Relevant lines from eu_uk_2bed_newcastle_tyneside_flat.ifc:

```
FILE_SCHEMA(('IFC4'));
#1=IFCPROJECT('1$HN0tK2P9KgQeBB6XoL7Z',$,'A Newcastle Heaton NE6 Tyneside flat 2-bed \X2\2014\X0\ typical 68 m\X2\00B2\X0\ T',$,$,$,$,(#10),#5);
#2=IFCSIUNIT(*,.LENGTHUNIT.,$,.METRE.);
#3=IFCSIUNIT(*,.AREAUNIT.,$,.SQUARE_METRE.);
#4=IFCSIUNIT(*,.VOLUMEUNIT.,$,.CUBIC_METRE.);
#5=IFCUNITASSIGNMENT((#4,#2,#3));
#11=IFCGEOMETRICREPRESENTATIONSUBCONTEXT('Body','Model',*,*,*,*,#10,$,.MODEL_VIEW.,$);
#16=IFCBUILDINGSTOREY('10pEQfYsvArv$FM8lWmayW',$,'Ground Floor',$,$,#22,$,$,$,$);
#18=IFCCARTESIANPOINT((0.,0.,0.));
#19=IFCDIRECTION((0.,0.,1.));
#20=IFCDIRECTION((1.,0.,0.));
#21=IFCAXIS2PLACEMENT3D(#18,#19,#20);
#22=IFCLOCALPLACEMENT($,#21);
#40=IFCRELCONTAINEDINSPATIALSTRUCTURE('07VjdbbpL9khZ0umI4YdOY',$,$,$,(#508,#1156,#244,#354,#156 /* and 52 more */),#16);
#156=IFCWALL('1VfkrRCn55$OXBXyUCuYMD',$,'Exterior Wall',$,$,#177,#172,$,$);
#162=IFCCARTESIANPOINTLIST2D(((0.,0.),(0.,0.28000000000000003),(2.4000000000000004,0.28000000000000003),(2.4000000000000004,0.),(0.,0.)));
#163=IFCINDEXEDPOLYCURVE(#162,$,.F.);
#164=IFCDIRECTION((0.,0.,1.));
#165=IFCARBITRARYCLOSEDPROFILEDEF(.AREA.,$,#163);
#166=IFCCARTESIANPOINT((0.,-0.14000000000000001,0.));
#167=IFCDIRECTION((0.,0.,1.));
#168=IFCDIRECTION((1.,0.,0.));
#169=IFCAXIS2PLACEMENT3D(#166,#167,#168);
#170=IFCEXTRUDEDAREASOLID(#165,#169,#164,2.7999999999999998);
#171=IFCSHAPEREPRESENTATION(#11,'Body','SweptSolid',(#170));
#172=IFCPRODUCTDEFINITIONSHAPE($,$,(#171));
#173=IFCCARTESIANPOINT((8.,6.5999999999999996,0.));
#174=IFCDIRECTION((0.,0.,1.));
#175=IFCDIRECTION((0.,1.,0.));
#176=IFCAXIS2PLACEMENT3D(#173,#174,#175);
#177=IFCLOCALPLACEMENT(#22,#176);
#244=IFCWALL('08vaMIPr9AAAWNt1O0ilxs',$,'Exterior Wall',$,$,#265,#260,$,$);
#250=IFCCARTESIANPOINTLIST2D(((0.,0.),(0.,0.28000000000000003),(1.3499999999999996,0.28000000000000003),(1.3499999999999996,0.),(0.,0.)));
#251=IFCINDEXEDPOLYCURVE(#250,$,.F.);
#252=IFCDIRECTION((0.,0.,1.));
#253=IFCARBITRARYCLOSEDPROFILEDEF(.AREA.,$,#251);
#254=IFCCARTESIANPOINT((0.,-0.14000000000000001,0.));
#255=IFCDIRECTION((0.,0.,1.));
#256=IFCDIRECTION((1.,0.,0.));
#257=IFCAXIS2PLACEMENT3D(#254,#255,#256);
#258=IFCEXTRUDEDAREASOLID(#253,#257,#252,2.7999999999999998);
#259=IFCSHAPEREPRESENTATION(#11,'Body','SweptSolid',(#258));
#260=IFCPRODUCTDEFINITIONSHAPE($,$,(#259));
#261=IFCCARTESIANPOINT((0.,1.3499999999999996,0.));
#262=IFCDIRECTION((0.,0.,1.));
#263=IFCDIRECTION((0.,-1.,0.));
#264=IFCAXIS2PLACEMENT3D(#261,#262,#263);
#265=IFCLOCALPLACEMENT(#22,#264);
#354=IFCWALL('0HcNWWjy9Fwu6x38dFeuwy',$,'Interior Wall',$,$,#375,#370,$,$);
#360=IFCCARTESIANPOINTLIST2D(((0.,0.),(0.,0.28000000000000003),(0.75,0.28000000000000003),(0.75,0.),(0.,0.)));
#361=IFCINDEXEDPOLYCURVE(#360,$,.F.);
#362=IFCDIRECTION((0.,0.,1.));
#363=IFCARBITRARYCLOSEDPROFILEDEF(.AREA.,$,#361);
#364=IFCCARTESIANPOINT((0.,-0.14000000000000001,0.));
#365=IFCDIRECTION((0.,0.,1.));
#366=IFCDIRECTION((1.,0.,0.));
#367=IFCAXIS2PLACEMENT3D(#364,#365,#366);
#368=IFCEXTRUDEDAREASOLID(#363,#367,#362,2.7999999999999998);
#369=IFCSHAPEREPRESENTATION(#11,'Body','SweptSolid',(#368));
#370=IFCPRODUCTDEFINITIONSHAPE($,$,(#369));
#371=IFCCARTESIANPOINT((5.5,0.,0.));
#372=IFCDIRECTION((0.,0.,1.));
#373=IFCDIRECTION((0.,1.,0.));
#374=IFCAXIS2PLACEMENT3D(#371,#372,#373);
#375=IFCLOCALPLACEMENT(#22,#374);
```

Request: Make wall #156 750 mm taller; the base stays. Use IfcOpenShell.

```python
import ifcopenshell
import ifcopenshell.geom
import ifcopenshell.util.representation
import ifcopenshell.util.shape

model = ifcopenshell.open("eu_uk_2bed_newcastle_tyneside_flat.ifc")
settings = ifcopenshell.geom.settings()


def volume(element):
    """Net volume in cubic metres, openings subtracted."""
    shape = ifcopenshell.geom.create_shape(settings, element)
    return ifcopenshell.util.shape.get_volume(shape.geometry)


wall = model.by_id(156)
before = volume(wall)

body = ifcopenshell.util.representation.get_representation(wall, "Model", "Body")
solid = body.Items[0]
old_height = solid.Depth
solid.Depth += 0.75
after = volume(wall)

print(f"height {old_height:g} -> {solid.Depth:g}, volume {before:.3f} -> {after:.3f} m3")

model.write("eu_uk_2bed_newcastle_tyneside_flat_v2.ifc")
```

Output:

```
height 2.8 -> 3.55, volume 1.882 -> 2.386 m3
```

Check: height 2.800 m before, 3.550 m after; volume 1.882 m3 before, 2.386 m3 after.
